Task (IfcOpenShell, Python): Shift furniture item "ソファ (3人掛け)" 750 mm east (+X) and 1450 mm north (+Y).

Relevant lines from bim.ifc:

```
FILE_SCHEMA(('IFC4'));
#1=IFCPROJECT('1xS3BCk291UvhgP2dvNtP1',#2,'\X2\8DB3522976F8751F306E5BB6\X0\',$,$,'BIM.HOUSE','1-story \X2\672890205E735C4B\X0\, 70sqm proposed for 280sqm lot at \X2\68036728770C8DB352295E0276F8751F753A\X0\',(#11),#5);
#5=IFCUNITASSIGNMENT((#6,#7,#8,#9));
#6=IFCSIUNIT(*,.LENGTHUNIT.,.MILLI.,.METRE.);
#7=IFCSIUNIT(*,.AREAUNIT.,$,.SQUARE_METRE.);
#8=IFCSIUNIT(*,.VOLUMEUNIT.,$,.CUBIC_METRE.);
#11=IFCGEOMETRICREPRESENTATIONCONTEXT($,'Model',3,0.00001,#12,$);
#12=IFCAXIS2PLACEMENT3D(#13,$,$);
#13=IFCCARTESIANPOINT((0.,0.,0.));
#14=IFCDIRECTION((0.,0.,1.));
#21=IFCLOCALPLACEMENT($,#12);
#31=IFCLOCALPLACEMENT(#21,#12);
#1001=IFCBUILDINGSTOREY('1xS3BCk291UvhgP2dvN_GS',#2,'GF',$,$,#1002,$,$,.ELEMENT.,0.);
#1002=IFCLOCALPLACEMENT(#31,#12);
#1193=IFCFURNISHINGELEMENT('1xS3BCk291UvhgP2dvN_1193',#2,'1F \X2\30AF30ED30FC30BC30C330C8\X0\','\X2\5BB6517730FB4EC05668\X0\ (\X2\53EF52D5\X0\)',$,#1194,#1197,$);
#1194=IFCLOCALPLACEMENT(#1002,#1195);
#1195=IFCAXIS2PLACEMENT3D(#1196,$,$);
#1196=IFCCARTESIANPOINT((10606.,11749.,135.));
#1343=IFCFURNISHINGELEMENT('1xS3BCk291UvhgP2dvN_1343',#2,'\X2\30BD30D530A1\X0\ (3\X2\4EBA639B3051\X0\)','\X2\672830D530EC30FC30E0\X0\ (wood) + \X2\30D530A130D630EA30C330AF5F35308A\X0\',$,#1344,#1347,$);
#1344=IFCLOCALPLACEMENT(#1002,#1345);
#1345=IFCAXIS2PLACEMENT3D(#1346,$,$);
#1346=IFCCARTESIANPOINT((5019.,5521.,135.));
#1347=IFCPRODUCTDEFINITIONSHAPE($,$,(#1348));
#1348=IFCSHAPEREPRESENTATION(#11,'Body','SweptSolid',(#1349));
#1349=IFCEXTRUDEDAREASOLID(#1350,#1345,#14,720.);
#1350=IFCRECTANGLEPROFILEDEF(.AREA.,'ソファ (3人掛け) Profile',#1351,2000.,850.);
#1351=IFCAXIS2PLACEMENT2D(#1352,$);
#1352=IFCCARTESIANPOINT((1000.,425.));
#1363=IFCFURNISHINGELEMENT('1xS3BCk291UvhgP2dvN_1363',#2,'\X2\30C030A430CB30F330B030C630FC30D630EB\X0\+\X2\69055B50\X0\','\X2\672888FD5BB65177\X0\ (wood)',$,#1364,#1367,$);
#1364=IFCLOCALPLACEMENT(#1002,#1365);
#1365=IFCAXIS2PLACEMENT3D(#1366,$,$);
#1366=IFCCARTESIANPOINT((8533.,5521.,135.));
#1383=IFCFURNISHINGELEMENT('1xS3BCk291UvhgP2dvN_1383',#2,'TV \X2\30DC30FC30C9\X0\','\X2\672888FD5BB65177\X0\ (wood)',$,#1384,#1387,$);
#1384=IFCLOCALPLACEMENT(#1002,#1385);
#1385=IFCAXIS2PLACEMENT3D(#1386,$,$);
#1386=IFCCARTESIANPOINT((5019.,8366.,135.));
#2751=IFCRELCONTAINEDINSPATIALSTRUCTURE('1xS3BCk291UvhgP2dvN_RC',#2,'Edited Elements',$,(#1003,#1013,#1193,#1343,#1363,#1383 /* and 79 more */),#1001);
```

```python
import ifcopenshell
import ifcopenshell.api.geometry
import ifcopenshell.util.placement

model = ifcopenshell.open("bim.ifc")

item = model.by_id(1343)
matrix = ifcopenshell.util.placement.get_local_placement(item.ObjectPlacement)
matrix[0, 3] += 750.0
matrix[1, 3] += 1450.0
ifcopenshell.api.geometry.edit_object_placement(model, product=item, matrix=matrix, is_si=False)

print(ifcopenshell.util.placement.get_local_placement(item.ObjectPlacement).round(3) + 0.0)

model.write("bim_v2.ifc")
```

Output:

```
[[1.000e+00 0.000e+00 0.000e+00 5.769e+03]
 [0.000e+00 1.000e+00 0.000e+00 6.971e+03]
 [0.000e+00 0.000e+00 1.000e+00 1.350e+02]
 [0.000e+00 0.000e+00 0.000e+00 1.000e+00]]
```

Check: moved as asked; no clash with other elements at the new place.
